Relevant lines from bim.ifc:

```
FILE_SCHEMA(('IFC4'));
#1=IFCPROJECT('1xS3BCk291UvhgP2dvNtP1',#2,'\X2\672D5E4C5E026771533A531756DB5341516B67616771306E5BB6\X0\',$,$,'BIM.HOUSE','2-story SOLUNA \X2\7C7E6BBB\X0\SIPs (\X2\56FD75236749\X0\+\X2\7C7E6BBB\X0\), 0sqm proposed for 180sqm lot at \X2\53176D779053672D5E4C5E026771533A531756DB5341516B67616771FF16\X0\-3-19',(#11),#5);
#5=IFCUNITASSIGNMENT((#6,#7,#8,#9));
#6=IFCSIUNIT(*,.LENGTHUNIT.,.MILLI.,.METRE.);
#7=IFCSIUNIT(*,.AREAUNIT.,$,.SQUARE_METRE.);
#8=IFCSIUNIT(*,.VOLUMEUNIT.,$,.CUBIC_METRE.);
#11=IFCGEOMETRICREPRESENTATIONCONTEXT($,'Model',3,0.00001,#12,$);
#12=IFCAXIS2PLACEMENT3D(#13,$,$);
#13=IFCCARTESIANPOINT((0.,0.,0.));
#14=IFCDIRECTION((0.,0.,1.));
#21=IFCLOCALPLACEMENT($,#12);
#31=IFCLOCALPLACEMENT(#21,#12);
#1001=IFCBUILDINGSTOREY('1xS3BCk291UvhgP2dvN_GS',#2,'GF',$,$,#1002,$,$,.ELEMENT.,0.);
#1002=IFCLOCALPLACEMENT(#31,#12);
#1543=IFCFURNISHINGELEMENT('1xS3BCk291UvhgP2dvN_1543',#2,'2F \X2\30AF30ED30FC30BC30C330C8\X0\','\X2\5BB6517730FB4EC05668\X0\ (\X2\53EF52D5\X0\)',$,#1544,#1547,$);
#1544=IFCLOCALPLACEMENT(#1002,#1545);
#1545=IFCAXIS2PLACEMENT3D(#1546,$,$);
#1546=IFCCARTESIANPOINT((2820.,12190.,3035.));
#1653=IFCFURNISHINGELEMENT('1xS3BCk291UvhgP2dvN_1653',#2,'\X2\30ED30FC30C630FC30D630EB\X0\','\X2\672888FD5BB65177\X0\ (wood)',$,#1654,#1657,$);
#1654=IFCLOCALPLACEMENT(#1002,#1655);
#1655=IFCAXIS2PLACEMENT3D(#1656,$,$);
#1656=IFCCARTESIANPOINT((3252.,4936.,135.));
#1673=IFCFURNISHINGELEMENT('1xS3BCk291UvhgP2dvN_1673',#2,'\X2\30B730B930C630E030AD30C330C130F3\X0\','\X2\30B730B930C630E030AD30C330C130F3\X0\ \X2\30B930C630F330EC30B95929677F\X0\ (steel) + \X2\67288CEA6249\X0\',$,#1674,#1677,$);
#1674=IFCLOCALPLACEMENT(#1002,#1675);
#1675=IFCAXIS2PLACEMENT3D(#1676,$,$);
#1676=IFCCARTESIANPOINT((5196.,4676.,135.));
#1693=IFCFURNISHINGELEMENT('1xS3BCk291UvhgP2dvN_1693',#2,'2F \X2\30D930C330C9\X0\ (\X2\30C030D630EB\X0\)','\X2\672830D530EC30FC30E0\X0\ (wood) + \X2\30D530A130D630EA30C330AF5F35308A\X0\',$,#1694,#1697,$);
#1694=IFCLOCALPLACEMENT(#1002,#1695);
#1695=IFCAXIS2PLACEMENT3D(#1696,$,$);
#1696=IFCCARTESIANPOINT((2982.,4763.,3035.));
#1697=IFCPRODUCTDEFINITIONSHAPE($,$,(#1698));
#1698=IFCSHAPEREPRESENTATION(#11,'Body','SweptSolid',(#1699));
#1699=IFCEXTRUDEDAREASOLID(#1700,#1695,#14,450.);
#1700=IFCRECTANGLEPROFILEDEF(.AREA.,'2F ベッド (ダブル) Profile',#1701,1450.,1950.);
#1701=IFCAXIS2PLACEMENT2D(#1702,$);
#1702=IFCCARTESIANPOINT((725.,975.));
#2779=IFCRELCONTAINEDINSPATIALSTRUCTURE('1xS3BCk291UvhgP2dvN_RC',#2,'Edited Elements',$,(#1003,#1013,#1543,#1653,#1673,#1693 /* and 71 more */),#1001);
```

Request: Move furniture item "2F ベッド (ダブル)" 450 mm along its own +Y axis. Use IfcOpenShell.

```python
import ifcopenshell
import ifcopenshell.api.geometry
import ifcopenshell.util.placement

model = ifcopenshell.open("bim.ifc")

item = model.by_guid("1xS3BCk291UvhgP2dvN_1693")
matrix = ifcopenshell.util.placement.get_local_placement(item.ObjectPlacement)
matrix[:3, 3] += matrix[:3, 1] * 450.0
ifcopenshell.api.geometry.edit_object_placement(model, product=item, matrix=matrix, is_si=False)

print(ifcopenshell.util.placement.get_local_placement(item.ObjectPlacement).round(3) + 0.0)

model.write("bim_updated.ifc")
```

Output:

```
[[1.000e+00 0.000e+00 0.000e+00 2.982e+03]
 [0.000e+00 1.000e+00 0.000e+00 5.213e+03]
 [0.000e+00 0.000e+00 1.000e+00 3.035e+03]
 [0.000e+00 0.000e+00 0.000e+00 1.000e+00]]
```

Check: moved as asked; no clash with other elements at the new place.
